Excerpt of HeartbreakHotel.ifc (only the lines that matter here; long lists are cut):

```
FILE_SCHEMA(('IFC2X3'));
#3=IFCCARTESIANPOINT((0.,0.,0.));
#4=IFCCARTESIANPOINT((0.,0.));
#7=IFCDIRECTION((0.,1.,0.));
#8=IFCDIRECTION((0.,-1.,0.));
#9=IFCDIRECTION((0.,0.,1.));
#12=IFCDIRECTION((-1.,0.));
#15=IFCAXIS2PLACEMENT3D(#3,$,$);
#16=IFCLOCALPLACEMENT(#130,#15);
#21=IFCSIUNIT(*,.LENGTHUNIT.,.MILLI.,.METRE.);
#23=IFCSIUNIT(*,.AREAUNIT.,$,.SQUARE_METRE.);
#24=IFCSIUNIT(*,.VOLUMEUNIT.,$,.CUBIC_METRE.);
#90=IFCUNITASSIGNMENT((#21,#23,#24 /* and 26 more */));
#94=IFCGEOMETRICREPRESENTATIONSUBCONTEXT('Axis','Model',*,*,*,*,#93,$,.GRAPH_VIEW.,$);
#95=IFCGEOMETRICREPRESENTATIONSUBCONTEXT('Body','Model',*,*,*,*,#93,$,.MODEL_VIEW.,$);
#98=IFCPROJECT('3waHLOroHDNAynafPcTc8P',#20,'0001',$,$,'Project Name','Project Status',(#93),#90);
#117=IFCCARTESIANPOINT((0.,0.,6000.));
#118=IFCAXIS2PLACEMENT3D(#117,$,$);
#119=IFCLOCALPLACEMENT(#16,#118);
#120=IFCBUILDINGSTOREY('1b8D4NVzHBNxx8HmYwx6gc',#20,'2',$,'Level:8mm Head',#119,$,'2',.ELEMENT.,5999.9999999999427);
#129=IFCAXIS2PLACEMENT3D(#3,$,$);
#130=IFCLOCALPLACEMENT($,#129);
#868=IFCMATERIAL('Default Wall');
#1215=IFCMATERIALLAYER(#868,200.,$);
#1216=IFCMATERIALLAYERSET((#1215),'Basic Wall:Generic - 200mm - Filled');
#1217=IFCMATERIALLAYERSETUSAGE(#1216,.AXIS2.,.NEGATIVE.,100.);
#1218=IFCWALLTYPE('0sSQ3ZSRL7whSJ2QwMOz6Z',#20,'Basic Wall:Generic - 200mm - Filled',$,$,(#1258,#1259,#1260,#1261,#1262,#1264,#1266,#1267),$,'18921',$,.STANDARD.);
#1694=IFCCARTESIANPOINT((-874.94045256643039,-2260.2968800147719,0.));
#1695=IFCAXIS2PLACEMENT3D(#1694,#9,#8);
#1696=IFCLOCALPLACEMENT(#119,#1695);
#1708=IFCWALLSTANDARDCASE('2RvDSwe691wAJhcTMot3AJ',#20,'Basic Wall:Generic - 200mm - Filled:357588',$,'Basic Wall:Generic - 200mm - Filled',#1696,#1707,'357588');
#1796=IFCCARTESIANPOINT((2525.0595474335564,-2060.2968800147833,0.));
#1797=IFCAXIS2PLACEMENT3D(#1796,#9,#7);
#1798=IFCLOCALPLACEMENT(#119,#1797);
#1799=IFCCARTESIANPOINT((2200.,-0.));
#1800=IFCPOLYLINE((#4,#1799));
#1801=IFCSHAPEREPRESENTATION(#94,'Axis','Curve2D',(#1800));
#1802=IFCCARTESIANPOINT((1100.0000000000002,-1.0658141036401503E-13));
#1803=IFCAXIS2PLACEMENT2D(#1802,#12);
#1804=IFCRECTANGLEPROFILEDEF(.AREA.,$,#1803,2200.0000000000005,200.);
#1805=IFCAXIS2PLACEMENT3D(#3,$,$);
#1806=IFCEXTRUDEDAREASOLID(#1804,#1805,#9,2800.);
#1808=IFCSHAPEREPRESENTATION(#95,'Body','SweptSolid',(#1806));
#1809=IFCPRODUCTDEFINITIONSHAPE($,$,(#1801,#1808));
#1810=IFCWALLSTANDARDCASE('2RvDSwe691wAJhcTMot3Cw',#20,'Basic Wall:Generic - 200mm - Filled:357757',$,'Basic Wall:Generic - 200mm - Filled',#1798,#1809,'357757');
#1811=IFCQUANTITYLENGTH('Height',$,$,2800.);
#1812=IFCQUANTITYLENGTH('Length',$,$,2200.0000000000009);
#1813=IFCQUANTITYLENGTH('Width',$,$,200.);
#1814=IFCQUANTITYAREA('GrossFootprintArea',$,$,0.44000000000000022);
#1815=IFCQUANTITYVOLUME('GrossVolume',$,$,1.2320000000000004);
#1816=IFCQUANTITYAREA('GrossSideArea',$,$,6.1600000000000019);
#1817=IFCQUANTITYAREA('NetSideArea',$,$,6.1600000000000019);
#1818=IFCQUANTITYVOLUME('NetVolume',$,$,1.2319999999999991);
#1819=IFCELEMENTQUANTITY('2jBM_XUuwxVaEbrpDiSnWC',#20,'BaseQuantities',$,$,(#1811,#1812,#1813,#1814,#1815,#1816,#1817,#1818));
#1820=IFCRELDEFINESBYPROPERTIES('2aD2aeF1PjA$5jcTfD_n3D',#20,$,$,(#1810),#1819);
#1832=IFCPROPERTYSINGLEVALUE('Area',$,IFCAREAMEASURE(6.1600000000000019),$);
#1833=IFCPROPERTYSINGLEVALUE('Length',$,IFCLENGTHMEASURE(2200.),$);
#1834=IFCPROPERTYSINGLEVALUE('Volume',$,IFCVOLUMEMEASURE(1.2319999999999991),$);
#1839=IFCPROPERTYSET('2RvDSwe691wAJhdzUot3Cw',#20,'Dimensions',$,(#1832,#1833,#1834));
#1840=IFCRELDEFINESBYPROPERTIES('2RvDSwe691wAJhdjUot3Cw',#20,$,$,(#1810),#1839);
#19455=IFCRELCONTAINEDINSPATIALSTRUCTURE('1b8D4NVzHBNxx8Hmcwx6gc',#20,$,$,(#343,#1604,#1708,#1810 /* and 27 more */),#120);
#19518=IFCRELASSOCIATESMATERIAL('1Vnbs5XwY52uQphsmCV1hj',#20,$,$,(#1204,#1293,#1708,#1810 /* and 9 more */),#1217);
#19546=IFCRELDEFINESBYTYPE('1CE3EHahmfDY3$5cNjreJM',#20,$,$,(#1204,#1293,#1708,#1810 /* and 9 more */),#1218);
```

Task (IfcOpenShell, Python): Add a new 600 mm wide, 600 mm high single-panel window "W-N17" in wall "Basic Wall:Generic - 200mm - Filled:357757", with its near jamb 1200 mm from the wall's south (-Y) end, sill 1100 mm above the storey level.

```python
import numpy as np
import ifcopenshell
import ifcopenshell.api.feature
import ifcopenshell.api.geometry
import ifcopenshell.api.pset
import ifcopenshell.api.root
import ifcopenshell.api.spatial
import ifcopenshell.api.type
import ifcopenshell.geom
import ifcopenshell.util.element
import ifcopenshell.util.placement
import ifcopenshell.util.representation
import ifcopenshell.util.shape
import ifcopenshell.util.unit

model = ifcopenshell.open("HeartbreakHotel.ifc")
unit_scale = ifcopenshell.util.unit.calculate_unit_scale(model)
area_scale = ifcopenshell.util.unit.calculate_unit_scale(model, "AREAUNIT")
volume_scale = ifcopenshell.util.unit.calculate_unit_scale(model, "VOLUMEUNIT")
settings = ifcopenshell.geom.settings()


def volume(element):
    """Net volume in cubic metres, openings subtracted."""
    shape = ifcopenshell.geom.create_shape(settings, element)
    return ifcopenshell.util.shape.get_volume(shape.geometry)


wall = model.by_id(1810)
storey = ifcopenshell.util.element.get_container(wall, ifc_class="IfcBuildingStorey")
context = ifcopenshell.util.representation.get_context(model, "Model", "Body", "MODEL_VIEW")
before = volume(wall)

width, height, from_end, sill = 0.6, 0.6, 1.2, 1.1  # metres

# The wall runs along its own X axis, and the end named is its -X end.
wall_shape = ifcopenshell.geom.create_shape(settings, wall)
x, y, z = ifcopenshell.util.shape.get_vertices(wall_shape.geometry).T
start = x.min() + from_end
face, thickness = float(y.min()), float(y.max() - y.min())
wall_matrix = ifcopenshell.util.placement.get_local_placement(wall.ObjectPlacement)
level = ifcopenshell.util.placement.get_local_placement(storey.ObjectPlacement)[2, 3]


def in_wall(x, y):
    """Placement at x, y metres in the wall's axes, at sill height."""
    matrix = wall_matrix.copy()
    matrix[:, 3] = wall_matrix @ np.array([x / unit_scale, y / unit_scale, 0.0, 1.0])
    matrix[2, 3] = level + sill / unit_scale
    return matrix


# Opening: a box that overshoots both wall faces by 50 mm.
opening = ifcopenshell.api.root.create_entity(model, ifc_class="IfcOpeningElement")
box = ifcopenshell.api.geometry.add_wall_representation(
    model, context=context, length=width, height=height, thickness=thickness + 0.1
)
ifcopenshell.api.geometry.assign_representation(model, product=opening, representation=box)
ifcopenshell.api.geometry.edit_object_placement(model, product=opening, matrix=in_wall(start, face - 0.05), is_si=False)
ifcopenshell.api.feature.add_feature(model, feature=opening, element=wall)

window = ifcopenshell.api.root.create_entity(model, ifc_class="IfcWindow", name="W-N17")
window.OverallWidth, window.OverallHeight = width / unit_scale, height / unit_scale
body = ifcopenshell.api.geometry.add_window_representation(
    model,
    context=context,
    overall_width=window.OverallWidth,
    overall_height=window.OverallHeight,
    partition_type="SINGLE_PANEL",
)
ifcopenshell.api.geometry.assign_representation(model, product=window, representation=body)
ifcopenshell.api.spatial.assign_container(model, products=[window], relating_structure=storey)
fills = ifcopenshell.api.feature.add_filling(model, opening=opening, element=window)
fills.OwnerHistory = window.OwnerHistory  # required in IFC2X3

# IFC2X3 keeps the operation on the window style.
style = ifcopenshell.api.root.create_entity(model, ifc_class="IfcWindowStyle", name="W-N17")
style.OperationType, style.ConstructionType = "SINGLE_PANEL", "NOTDEFINED"
style.ParameterTakesPrecedence = style.Sizeable = False
ifcopenshell.api.type.assign_type(model, related_objects=[window], relating_type=style)

# Centre the window in the wall's thickness.
ifcopenshell.api.geometry.edit_object_placement(model, product=window, matrix=in_wall(start, face), is_si=False)
window_shape = ifcopenshell.geom.create_shape(settings, window)
depth = ifcopenshell.util.shape.get_vertices(window_shape.geometry)[:, 1]
offset = face + thickness / 2 - (depth.min() + depth.max()) / 2
ifcopenshell.api.geometry.edit_object_placement(model, product=window, matrix=in_wall(start, offset), is_si=False)

after = volume(wall)

# Update the wall's stored quantities.
qto = model.by_id(ifcopenshell.util.element.get_pset(wall, "BaseQuantities", should_inherit=False)["id"])
ifcopenshell.api.pset.edit_qto(model, qto=qto, properties={
    "NetSideArea": after / thickness / area_scale,
    "NetVolume": after / volume_scale,
})
pset = model.by_id(ifcopenshell.util.element.get_pset(wall, "Dimensions", should_inherit=False)["id"])
ifcopenshell.api.pset.edit_pset(model, pset=pset, properties={
    "Area": model.create_entity("IfcAreaMeasure", after / thickness / area_scale),
    "Volume": model.create_entity("IfcVolumeMeasure", after / volume_scale),
})

print(f"wall volume {before:.3f} -> {after:.3f} m3")

model.write("HeartbreakHotel_rev.ifc")
```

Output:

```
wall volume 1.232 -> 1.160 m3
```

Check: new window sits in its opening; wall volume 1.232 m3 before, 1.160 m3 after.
